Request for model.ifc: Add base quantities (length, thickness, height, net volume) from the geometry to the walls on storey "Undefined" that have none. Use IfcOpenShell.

First a look at what the model holds.

```python
import ifcopenshell
import ifcopenshell.util.element
import ifcopenshell.util.unit

model = ifcopenshell.open("model.ifc")
print(model.schema)
for unit_type in ("LENGTHUNIT", "AREAUNIT", "VOLUMEUNIT"):
    print(unit_type, ifcopenshell.util.unit.calculate_unit_scale(model, unit_type))
storey = next(s for s in model.by_type("IfcBuildingStorey") if s.Name == "Undefined")
walls = [e for e in ifcopenshell.util.element.get_decomposition(storey) if e.is_a("IfcWall")]
for e in sorted(walls, key=lambda e: e.id()):
    print(e.id(), e.is_a(), e.Name, list(ifcopenshell.util.element.get_psets(e, qtos_only=True)), sep=" | ")
```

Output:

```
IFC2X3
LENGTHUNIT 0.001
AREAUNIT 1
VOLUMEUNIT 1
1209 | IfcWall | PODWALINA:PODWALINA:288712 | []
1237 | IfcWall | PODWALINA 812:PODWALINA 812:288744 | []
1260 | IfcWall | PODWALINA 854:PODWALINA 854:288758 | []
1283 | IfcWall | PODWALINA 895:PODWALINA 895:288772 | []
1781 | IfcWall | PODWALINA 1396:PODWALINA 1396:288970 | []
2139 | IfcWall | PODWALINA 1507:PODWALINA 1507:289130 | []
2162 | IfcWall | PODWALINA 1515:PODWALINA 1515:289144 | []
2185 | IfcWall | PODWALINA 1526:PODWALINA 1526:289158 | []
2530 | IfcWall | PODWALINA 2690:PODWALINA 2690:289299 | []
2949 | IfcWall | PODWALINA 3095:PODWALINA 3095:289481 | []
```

```python
import ifcopenshell
import ifcopenshell.api.pset
import ifcopenshell.geom
import ifcopenshell.util.element
import ifcopenshell.util.shape
import ifcopenshell.util.unit

model = ifcopenshell.open("model.ifc")
unit_scale = ifcopenshell.util.unit.calculate_unit_scale(model)
volume_scale = ifcopenshell.util.unit.calculate_unit_scale(model, "VOLUMEUNIT")
settings = ifcopenshell.geom.settings()

storey = next(s for s in model.by_type("IfcBuildingStorey") if s.Name == "Undefined")
walls = [e for e in ifcopenshell.util.element.get_decomposition(storey) if e.is_a("IfcWall")]

for e in sorted(walls, key=lambda e: e.id()):
    if ifcopenshell.util.element.get_psets(e, qtos_only=True, should_inherit=False):
        continue
    # Geometry comes back in metres, in the element's own axes.
    shape = ifcopenshell.geom.create_shape(settings, e)
    values = {
        "Length": ifcopenshell.util.shape.get_x(shape.geometry) / unit_scale,
        "Width": ifcopenshell.util.shape.get_y(shape.geometry) / unit_scale,
        "Height": ifcopenshell.util.shape.get_z(shape.geometry) / unit_scale,
        "NetVolume": ifcopenshell.util.shape.get_volume(shape.geometry) / volume_scale,
    }
    qto = ifcopenshell.api.pset.add_qto(model, product=e, name="BaseQuantities")
    ifcopenshell.api.pset.edit_qto(model, qto=qto, properties=values)
    print(e.id(), {k: round(v, 3) for k, v in values.items()})

model.write("model_updated.ifc")
```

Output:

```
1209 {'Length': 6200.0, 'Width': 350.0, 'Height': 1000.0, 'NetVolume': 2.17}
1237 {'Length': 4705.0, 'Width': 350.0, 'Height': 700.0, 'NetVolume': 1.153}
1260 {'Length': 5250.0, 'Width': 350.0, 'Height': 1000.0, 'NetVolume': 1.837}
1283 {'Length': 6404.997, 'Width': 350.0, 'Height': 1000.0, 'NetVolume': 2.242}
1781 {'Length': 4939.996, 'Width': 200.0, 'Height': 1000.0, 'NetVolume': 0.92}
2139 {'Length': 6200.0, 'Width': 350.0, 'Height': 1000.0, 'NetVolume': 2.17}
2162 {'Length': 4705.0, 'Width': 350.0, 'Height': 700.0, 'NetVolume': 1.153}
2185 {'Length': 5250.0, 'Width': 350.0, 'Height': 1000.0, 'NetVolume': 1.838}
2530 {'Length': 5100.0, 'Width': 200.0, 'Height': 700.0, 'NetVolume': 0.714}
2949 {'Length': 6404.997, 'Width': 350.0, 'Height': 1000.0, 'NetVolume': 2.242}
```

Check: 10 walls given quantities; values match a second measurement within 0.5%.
